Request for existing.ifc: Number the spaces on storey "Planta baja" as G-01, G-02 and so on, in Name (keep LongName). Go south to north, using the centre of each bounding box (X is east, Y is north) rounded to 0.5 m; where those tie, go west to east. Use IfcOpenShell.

First a look at what the model holds.

```python
import ifcopenshell
import ifcopenshell.util.element
import ifcopenshell.util.placement

model = ifcopenshell.open("existing.ifc")
print(model.schema)
storey = next(s for s in model.by_type("IfcBuildingStorey") if s.Name == "Planta baja")
spaces = [e for e in ifcopenshell.util.element.get_decomposition(storey) if e.is_a("IfcSpace")]
for e in sorted(spaces, key=lambda e: e.id()):
    origin = ifcopenshell.util.placement.get_local_placement(e.ObjectPlacement)[:3, 3]
    print(e.id(), e.Name, e.LongName, origin.round(2) + 0.0, sep=" | ")
```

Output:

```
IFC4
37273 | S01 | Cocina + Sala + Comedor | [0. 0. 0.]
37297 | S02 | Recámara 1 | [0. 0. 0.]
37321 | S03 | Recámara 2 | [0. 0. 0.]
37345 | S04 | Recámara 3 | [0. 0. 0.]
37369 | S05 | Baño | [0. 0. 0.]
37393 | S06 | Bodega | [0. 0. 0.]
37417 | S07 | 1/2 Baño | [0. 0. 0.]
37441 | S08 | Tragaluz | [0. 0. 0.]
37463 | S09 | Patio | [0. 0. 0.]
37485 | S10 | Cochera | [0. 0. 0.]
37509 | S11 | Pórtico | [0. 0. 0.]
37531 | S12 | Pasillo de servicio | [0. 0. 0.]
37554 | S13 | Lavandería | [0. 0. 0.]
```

```python
import ifcopenshell
import ifcopenshell.geom
import ifcopenshell.util.element
import ifcopenshell.util.shape

model = ifcopenshell.open("existing.ifc")
settings = ifcopenshell.geom.settings()
settings.set("use-world-coords", True)


def centre(element):
    shape = ifcopenshell.geom.create_shape(settings, element)
    return ifcopenshell.util.shape.get_bbox_centroid(shape.geometry)


storey = next(s for s in model.by_type("IfcBuildingStorey") if s.Name == "Planta baja")
spaces = [e for e in ifcopenshell.util.element.get_decomposition(storey) if e.is_a("IfcSpace")]

# Insertion points can sit at a corner or the storey origin, so sort by the geometry (in metres).
centres = {e: centre(e) for e in spaces}
spaces.sort(key=lambda e: (round(centres[e][1] / 0.5), centres[e][0]))

for i, e in enumerate(spaces, start=1):
    number = f"G-{i:02d}"
    e.Name = number
    print(e.id(), number)

model.write("existing_rev.ifc")
```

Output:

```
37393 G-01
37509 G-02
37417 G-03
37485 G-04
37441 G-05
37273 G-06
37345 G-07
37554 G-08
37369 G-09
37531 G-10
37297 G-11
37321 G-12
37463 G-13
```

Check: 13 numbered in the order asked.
